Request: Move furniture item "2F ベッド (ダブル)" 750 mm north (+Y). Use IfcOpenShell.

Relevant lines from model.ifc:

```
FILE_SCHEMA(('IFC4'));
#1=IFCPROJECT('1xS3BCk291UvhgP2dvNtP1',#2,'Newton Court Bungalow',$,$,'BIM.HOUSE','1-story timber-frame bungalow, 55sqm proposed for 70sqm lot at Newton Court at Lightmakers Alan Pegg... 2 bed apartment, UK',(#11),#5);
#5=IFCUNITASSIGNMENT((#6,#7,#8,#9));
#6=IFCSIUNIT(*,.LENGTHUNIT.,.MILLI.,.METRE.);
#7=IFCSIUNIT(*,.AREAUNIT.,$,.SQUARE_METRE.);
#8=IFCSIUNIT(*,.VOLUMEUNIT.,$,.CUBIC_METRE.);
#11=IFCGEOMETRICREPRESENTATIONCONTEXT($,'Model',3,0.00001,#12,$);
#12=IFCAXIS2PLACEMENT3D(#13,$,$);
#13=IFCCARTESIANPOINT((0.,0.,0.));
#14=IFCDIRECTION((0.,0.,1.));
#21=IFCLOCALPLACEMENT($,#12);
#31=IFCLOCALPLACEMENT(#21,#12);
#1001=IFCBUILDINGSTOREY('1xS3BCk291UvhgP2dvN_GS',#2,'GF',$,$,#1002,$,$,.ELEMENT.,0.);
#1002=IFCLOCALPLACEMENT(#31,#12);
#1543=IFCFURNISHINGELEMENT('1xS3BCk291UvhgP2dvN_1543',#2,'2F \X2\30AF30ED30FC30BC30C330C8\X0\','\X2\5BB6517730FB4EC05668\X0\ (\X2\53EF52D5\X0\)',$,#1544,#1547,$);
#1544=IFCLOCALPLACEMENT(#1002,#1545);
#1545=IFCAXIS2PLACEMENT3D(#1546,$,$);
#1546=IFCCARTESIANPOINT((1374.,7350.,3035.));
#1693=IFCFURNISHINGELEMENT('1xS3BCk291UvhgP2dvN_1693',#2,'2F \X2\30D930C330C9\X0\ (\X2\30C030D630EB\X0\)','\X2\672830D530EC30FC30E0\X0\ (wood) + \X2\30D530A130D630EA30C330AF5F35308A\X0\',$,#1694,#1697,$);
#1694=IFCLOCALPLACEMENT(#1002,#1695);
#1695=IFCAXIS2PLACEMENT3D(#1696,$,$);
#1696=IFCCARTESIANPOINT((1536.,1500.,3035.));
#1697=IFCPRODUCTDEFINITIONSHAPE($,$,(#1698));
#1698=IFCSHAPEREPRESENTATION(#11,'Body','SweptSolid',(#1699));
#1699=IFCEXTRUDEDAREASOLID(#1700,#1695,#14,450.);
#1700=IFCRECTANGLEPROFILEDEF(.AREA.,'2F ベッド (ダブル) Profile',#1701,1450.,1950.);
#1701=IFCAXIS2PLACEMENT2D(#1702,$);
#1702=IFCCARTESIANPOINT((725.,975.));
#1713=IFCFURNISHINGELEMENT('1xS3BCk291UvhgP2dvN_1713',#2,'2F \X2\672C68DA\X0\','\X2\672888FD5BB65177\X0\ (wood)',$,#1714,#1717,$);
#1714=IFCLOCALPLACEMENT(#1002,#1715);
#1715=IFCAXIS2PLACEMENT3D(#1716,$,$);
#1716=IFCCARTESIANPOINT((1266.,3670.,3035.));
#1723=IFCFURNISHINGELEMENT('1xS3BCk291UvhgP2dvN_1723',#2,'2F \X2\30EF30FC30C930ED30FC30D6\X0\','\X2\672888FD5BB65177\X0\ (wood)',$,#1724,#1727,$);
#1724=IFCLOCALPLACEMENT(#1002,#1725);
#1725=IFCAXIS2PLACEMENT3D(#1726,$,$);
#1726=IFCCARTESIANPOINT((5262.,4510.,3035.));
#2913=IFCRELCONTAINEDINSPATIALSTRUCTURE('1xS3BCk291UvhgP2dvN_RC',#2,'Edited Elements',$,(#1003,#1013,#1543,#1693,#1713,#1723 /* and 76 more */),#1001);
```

```python
import ifcopenshell
import ifcopenshell.api.geometry
import ifcopenshell.util.placement
import ifcopenshell.util.unit

model = ifcopenshell.open("model.ifc")
unit_scale = ifcopenshell.util.unit.calculate_unit_scale(model)

item = model.by_guid("1xS3BCk291UvhgP2dvN_1693")
matrix = ifcopenshell.util.placement.get_local_placement(item.ObjectPlacement)
matrix[1, 3] += 0.75 / unit_scale
ifcopenshell.api.geometry.edit_object_placement(model, product=item, matrix=matrix, is_si=False)

print(ifcopenshell.util.placement.get_local_placement(item.ObjectPlacement).round(3) + 0.0)

model.write("model-out.ifc")
```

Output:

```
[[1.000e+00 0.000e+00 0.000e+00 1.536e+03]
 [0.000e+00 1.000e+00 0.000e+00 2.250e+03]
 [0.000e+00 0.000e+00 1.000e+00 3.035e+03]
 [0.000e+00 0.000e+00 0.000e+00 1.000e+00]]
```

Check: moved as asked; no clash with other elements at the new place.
